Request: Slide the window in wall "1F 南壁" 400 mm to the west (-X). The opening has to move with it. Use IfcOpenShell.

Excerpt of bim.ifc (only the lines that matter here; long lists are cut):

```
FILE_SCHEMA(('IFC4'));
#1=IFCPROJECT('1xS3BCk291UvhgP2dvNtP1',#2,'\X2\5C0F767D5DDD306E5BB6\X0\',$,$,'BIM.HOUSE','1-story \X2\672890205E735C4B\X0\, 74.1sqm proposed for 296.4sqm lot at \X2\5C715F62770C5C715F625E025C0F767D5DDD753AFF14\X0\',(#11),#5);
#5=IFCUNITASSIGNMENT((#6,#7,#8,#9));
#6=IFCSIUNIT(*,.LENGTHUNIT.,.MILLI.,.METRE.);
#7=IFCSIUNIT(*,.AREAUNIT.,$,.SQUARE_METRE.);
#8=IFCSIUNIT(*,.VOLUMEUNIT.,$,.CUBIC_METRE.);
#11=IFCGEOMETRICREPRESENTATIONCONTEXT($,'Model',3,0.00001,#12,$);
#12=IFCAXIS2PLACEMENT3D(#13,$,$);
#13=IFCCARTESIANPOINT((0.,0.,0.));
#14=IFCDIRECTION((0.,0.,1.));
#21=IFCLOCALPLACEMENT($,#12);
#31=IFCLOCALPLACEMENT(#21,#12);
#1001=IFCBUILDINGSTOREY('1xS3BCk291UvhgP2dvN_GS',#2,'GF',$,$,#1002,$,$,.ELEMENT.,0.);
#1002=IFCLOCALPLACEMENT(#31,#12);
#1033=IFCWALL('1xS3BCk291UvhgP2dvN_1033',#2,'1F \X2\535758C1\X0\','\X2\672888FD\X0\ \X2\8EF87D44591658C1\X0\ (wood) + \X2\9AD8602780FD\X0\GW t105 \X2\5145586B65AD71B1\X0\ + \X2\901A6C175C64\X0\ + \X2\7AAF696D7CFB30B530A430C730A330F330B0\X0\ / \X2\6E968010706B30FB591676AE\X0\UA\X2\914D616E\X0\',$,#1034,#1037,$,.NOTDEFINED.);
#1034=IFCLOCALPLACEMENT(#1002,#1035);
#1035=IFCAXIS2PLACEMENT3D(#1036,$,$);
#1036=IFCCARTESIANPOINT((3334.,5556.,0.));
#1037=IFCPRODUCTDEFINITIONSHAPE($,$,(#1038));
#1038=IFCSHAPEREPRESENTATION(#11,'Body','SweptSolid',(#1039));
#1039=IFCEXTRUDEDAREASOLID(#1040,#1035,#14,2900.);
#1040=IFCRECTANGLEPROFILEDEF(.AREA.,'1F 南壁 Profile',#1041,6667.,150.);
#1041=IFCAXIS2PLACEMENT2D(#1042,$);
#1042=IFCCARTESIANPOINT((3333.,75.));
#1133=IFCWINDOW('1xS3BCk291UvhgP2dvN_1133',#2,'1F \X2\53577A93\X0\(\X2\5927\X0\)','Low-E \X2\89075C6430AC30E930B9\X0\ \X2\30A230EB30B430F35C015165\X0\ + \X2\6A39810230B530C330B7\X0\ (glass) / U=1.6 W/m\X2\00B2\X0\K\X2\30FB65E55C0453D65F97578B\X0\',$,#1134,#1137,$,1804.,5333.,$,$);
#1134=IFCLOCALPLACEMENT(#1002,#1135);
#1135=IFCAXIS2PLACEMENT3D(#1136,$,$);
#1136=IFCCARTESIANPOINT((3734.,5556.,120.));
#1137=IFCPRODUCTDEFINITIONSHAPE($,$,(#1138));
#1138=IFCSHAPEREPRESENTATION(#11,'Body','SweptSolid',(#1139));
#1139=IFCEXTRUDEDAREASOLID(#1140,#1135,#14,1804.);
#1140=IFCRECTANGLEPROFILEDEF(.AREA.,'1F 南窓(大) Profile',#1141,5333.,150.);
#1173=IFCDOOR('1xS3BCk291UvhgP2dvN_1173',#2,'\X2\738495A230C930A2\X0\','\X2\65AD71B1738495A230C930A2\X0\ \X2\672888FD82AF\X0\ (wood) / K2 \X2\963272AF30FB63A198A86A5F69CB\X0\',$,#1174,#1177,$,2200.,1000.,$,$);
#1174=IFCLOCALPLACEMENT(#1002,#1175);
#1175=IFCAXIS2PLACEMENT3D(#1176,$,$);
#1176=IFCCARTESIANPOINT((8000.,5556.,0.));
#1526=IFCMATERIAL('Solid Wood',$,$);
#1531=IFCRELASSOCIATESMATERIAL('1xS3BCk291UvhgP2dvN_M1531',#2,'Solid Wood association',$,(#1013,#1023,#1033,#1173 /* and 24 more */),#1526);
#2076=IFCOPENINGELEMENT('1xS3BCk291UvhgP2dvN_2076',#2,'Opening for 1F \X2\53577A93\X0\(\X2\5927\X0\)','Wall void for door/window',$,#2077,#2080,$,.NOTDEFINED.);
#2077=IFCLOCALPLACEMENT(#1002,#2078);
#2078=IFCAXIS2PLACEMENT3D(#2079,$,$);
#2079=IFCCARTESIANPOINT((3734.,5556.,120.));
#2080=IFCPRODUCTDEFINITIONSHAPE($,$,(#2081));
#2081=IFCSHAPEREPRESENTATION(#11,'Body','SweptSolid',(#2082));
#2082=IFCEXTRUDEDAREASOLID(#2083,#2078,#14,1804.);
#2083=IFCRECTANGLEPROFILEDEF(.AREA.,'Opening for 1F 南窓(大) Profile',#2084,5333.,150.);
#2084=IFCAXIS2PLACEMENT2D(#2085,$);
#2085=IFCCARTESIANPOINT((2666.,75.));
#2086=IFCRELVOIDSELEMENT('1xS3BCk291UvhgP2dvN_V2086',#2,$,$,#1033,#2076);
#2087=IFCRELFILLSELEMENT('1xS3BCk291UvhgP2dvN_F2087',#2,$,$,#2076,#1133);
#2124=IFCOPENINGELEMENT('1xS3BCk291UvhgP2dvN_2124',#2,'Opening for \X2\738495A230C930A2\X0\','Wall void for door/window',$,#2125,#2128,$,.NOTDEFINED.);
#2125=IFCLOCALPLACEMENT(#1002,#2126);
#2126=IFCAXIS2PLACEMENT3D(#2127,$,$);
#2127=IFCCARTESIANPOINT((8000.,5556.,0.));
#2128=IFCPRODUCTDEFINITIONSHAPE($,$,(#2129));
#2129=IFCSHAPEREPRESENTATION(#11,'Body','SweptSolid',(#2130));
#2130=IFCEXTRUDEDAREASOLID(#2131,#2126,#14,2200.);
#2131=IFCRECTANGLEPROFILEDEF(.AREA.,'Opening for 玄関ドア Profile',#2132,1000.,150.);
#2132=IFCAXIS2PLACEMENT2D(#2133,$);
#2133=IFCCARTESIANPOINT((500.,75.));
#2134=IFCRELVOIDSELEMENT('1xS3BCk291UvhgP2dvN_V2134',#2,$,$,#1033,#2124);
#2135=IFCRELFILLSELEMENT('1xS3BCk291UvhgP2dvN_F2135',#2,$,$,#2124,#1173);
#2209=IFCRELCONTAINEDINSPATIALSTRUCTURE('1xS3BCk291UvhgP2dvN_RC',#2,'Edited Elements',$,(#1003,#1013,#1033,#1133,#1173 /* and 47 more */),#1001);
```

```python
import ifcopenshell
import ifcopenshell.api.geometry
import ifcopenshell.util.placement
import ifcopenshell.util.unit

model = ifcopenshell.open("bim.ifc")
unit_scale = ifcopenshell.util.unit.calculate_unit_scale(model)

window = model.by_id(1133)
opening = window.FillsVoids[0].RelatingOpeningElement
wall = opening.VoidsElements[0].RelatingBuildingElement

wall_matrix = ifcopenshell.util.placement.get_local_placement(wall.ObjectPlacement)
shift = wall_matrix[:3, 0] * -0.4 / unit_scale
before = ifcopenshell.util.placement.get_local_placement(window.ObjectPlacement)[:3, 3].copy()

# The window is not placed relative to its opening, so move both.
for product in (opening, window):
    matrix = ifcopenshell.util.placement.get_local_placement(product.ObjectPlacement)
    matrix[:3, 3] += shift
    ifcopenshell.api.geometry.edit_object_placement(model, product=product, matrix=matrix, is_si=False)

after = ifcopenshell.util.placement.get_local_placement(window.ObjectPlacement)[:3, 3]
print("window moved by", (after - before).round(3) + 0.0)

model.write("bim_edited.ifc")
```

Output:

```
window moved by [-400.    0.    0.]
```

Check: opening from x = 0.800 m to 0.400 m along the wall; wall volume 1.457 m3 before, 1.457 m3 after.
